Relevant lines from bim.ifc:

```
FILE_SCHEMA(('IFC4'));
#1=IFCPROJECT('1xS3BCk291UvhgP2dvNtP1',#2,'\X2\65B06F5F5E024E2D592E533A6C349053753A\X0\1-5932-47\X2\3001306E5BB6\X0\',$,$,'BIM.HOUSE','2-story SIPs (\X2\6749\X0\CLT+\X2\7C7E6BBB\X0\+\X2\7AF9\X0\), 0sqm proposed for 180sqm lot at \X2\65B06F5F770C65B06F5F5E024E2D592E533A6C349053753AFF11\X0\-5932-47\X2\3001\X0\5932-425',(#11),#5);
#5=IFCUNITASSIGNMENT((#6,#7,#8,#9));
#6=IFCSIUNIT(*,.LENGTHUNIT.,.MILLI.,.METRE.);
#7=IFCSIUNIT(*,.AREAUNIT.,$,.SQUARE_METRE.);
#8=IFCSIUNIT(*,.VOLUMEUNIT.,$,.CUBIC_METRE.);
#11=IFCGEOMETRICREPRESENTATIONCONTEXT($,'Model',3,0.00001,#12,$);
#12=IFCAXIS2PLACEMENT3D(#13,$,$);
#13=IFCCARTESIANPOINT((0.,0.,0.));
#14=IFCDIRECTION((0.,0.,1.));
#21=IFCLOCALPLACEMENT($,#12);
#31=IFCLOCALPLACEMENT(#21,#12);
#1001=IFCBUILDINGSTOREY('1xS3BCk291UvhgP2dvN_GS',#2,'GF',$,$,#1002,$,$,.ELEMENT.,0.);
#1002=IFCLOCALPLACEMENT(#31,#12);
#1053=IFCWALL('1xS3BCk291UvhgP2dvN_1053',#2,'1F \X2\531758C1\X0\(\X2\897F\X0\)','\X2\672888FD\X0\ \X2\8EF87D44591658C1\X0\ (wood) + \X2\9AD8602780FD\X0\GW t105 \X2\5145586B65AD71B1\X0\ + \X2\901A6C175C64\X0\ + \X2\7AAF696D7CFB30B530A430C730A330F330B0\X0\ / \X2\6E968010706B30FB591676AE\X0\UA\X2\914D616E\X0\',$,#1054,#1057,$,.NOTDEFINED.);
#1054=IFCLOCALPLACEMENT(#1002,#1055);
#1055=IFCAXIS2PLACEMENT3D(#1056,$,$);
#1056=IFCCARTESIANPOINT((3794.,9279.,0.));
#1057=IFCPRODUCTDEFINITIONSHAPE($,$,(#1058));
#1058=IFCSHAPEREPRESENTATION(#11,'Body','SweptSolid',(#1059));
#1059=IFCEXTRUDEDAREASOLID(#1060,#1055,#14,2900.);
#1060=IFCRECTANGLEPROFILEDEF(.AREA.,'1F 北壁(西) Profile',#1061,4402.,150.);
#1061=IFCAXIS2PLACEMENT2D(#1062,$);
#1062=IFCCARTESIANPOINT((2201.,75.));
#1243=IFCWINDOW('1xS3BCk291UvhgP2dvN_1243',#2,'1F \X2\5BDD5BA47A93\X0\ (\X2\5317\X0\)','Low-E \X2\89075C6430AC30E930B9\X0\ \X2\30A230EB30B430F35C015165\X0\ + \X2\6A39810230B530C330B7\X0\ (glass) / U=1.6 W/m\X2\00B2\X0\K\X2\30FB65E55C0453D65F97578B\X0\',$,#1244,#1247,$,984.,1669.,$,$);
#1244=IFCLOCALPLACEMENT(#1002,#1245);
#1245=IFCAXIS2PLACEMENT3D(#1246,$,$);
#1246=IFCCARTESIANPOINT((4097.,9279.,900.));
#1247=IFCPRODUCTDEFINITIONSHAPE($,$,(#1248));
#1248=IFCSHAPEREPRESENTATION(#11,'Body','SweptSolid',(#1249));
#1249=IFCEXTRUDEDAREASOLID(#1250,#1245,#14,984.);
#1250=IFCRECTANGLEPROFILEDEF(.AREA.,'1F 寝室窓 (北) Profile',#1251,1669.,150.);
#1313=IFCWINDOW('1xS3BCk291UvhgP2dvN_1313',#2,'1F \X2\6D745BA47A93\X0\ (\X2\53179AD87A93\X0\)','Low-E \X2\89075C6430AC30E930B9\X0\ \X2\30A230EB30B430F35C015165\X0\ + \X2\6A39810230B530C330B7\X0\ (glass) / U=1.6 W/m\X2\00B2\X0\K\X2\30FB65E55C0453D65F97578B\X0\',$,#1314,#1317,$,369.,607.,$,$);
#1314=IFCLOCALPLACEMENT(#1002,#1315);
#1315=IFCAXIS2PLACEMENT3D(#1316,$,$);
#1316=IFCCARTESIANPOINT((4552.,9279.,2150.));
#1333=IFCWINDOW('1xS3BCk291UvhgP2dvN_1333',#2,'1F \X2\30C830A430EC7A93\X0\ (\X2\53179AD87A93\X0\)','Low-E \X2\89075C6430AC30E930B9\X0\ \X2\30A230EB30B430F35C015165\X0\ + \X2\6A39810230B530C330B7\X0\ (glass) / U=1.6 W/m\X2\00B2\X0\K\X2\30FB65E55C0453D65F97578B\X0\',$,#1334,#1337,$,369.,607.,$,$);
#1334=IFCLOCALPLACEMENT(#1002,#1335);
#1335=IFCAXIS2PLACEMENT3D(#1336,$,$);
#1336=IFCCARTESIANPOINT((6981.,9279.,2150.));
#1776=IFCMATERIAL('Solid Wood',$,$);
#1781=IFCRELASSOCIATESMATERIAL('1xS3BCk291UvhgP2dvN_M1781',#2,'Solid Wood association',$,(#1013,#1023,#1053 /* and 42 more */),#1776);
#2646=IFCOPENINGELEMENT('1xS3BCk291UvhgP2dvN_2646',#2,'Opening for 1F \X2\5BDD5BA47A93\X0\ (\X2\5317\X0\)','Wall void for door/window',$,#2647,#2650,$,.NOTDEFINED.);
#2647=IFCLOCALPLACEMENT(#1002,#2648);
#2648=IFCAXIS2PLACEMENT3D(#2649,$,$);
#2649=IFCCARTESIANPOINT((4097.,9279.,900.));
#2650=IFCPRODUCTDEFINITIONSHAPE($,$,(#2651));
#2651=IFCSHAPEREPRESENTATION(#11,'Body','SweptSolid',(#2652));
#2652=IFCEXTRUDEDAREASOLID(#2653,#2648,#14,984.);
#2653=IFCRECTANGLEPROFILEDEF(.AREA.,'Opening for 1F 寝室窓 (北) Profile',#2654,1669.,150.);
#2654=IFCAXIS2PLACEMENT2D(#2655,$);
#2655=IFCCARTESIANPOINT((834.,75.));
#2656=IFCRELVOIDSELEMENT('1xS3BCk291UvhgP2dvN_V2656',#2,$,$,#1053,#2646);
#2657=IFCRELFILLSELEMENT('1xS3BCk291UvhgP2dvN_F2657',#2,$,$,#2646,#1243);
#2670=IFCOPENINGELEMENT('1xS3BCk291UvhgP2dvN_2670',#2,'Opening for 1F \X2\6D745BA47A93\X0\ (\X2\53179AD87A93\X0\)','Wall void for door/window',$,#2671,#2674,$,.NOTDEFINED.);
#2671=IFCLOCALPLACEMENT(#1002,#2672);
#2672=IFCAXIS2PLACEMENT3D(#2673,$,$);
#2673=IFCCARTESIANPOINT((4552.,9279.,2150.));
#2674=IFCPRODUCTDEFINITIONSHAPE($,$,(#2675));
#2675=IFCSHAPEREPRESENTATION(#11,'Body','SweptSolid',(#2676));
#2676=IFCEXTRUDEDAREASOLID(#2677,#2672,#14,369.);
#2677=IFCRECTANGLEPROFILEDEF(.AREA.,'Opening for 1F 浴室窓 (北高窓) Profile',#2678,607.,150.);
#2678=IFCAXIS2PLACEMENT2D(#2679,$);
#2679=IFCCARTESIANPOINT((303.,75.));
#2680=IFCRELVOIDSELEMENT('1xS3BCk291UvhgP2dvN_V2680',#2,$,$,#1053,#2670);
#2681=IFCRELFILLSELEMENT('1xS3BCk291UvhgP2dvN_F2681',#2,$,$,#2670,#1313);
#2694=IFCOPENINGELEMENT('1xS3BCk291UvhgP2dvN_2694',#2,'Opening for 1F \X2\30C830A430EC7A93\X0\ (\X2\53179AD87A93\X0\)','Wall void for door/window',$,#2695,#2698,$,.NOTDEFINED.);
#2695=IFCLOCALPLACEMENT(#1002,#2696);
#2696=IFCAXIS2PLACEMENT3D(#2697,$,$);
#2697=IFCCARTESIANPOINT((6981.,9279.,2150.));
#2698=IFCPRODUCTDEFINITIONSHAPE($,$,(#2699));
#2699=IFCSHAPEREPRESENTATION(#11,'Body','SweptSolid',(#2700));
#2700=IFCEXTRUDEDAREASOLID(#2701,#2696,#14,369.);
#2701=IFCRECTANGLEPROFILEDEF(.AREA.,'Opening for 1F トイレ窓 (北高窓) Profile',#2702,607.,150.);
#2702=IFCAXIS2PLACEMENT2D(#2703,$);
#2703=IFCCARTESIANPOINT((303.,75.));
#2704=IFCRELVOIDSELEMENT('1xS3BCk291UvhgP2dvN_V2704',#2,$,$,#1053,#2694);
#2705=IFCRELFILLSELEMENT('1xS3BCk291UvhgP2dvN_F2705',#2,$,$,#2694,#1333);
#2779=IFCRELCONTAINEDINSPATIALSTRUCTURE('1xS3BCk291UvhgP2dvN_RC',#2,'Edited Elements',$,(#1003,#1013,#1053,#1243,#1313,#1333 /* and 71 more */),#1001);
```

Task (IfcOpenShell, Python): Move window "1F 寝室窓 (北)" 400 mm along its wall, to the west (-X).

```python
import ifcopenshell
import ifcopenshell.api.geometry
import ifcopenshell.util.placement
import ifcopenshell.util.unit

model = ifcopenshell.open("bim.ifc")
unit_scale = ifcopenshell.util.unit.calculate_unit_scale(model)

window = model.by_guid("1xS3BCk291UvhgP2dvN_1243")
opening = window.FillsVoids[0].RelatingOpeningElement
wall = opening.VoidsElements[0].RelatingBuildingElement

wall_matrix = ifcopenshell.util.placement.get_local_placement(wall.ObjectPlacement)
shift = wall_matrix[:3, 0] * -0.4 / unit_scale
before = ifcopenshell.util.placement.get_local_placement(window.ObjectPlacement)[:3, 3].copy()

# The window is not placed relative to its opening, so move both.
for product in (opening, window):
    matrix = ifcopenshell.util.placement.get_local_placement(product.ObjectPlacement)
    matrix[:3, 3] += shift
    ifcopenshell.api.geometry.edit_object_placement(model, product=product, matrix=matrix, is_si=False)

after = ifcopenshell.util.placement.get_local_placement(window.ObjectPlacement)[:3, 3]
print("window moved by", (after - before).round(3) + 0.0)

model.write("bim_updated.ifc")
```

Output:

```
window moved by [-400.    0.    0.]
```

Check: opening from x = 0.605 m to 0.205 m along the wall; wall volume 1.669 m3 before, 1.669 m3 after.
